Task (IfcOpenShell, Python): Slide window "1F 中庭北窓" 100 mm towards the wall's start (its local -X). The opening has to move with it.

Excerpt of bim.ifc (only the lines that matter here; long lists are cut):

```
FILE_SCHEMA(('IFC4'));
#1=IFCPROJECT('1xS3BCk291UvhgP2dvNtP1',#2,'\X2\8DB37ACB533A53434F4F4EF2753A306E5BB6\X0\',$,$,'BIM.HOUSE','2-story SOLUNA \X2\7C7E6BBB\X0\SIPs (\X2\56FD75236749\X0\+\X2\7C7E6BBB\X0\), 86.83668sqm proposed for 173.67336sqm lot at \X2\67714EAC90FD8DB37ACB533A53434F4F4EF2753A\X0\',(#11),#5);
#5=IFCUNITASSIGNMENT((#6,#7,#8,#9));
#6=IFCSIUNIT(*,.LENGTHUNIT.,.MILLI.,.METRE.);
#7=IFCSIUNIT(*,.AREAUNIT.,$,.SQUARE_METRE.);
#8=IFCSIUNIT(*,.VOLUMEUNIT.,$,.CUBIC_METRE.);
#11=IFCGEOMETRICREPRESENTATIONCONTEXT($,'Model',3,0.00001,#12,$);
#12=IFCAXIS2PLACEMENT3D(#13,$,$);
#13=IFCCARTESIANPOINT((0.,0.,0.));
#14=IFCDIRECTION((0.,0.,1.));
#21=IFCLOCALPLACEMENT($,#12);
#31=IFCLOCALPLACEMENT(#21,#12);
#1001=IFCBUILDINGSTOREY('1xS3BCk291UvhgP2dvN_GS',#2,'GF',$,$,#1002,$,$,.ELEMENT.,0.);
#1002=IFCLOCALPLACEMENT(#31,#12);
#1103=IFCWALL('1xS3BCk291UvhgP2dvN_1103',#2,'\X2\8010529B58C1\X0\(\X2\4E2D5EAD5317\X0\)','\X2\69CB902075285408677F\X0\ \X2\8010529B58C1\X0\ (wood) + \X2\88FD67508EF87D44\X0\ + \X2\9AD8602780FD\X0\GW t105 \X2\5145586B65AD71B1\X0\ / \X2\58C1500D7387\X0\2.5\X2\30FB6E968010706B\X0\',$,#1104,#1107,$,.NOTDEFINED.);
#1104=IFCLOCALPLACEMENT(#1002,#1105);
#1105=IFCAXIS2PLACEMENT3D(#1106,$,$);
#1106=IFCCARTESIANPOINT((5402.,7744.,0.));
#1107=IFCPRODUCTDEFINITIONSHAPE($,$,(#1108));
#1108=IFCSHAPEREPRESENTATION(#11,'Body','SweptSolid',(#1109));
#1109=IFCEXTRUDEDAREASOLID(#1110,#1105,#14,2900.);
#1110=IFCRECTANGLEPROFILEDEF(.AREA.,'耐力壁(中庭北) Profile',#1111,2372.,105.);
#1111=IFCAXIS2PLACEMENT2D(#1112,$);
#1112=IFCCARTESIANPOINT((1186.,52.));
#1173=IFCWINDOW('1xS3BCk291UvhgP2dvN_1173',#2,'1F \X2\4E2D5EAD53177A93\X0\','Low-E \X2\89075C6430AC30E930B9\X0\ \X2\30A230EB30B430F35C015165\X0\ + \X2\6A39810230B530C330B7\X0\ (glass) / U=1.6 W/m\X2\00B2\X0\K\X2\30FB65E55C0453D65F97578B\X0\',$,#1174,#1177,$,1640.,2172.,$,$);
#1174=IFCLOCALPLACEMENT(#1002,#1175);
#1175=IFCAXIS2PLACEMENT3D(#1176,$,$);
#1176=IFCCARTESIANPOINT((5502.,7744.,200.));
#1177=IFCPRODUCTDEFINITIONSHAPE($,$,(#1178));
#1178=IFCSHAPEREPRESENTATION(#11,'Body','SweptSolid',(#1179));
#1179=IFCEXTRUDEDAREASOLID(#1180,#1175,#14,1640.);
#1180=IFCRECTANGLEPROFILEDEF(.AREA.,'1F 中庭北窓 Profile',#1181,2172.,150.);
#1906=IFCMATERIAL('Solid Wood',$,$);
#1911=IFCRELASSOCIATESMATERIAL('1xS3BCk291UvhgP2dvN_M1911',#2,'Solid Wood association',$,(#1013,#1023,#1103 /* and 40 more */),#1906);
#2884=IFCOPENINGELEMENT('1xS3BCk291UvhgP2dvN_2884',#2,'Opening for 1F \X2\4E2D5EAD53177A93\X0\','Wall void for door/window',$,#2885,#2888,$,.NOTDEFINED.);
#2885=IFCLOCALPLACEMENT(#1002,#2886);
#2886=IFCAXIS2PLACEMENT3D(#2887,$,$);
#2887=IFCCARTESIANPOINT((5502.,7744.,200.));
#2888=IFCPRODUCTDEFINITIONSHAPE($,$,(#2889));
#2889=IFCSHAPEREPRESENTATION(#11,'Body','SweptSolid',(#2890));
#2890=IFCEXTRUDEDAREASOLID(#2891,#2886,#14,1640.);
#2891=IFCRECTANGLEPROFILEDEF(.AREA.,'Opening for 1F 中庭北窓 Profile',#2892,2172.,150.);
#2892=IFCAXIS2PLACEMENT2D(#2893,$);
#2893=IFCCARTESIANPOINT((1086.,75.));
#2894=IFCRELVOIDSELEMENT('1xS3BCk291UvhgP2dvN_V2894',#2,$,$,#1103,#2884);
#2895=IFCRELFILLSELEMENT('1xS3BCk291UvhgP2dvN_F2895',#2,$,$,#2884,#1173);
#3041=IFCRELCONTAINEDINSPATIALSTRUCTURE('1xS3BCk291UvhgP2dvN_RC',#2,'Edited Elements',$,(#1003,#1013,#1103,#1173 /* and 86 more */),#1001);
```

```python
import ifcopenshell
import ifcopenshell.api.geometry
import ifcopenshell.util.placement
import ifcopenshell.util.unit

model = ifcopenshell.open("bim.ifc")
unit_scale = ifcopenshell.util.unit.calculate_unit_scale(model)

window = model.by_id(1173)
opening = window.FillsVoids[0].RelatingOpeningElement
wall = opening.VoidsElements[0].RelatingBuildingElement

wall_matrix = ifcopenshell.util.placement.get_local_placement(wall.ObjectPlacement)
shift = wall_matrix[:3, 0] * -0.1 / unit_scale
before = ifcopenshell.util.placement.get_local_placement(window.ObjectPlacement)[:3, 3].copy()

# The window is not placed relative to its opening, so move both.
for product in (opening, window):
    matrix = ifcopenshell.util.placement.get_local_placement(product.ObjectPlacement)
    matrix[:3, 3] += shift
    ifcopenshell.api.geometry.edit_object_placement(model, product=product, matrix=matrix, is_si=False)

after = ifcopenshell.util.placement.get_local_placement(window.ObjectPlacement)[:3, 3]
print("window moved by", (after - before).round(3) + 0.0)

model.write("bim_updated.ifc")
```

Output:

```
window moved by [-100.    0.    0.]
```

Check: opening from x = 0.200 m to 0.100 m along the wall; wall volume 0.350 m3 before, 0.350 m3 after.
